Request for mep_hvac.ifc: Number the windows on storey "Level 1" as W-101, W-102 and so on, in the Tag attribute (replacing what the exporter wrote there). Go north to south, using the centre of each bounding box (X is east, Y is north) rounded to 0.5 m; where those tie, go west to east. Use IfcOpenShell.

First a look at what the model holds.

```python
import ifcopenshell
import ifcopenshell.util.element
import ifcopenshell.util.placement

model = ifcopenshell.open("mep_hvac.ifc")
print(model.schema)
storey = next(s for s in model.by_type("IfcBuildingStorey") if s.Name == "Level 1")
windows = [e for e in ifcopenshell.util.element.get_decomposition(storey) if e.is_a("IfcWindow")]
for e in sorted(windows, key=lambda e: e.id()):
    origin = ifcopenshell.util.placement.get_local_placement(e.ObjectPlacement)[:3, 3]
    print(e.id(), e.Tag, e.Name, origin.round(2) + 0.0, sep=" | ")
```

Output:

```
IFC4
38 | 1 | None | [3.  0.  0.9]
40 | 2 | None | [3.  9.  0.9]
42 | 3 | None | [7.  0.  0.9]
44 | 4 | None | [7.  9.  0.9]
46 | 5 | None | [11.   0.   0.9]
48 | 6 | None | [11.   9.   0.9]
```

```python
import ifcopenshell
import ifcopenshell.geom
import ifcopenshell.util.element
import ifcopenshell.util.shape

model = ifcopenshell.open("mep_hvac.ifc")
settings = ifcopenshell.geom.settings()
settings.set("use-world-coords", True)


def centre(element):
    shape = ifcopenshell.geom.create_shape(settings, element)
    return ifcopenshell.util.shape.get_bbox_centroid(shape.geometry)


storey = next(s for s in model.by_type("IfcBuildingStorey") if s.Name == "Level 1")
windows = [e for e in ifcopenshell.util.element.get_decomposition(storey) if e.is_a("IfcWindow")]

# Insertion points can sit at a corner or the storey origin, so sort by the geometry (in metres).
centres = {e: centre(e) for e in windows}
windows.sort(key=lambda e: (-round(centres[e][1] / 0.5), centres[e][0]))

for i, e in enumerate(windows, start=1):
    number = f"W-1{i:02d}"
    e.Tag = number
    print(e.id(), number)

model.write("mep_hvac-out.ifc")
```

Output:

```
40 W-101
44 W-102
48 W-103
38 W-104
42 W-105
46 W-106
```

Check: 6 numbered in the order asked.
